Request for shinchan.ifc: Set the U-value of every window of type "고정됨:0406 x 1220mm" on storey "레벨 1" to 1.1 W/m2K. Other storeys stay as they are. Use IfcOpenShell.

First a look at what the model holds.

```python
import ifcopenshell
import ifcopenshell.util.element

model = ifcopenshell.open("shinchan.ifc")
print(model.schema)
storey = next(s for s in model.by_type("IfcBuildingStorey") if s.Name == "레벨 1")
windows = [e for e in ifcopenshell.util.element.get_decomposition(storey) if e.is_a("IfcWindow")]
seen = {}
for e in windows:
    element_type = ifcopenshell.util.element.get_type(e)
    key = (element_type.Name if element_type != e and element_type else None, ifcopenshell.util.element.get_pset(e, "Pset_WindowCommon", "ThermalTransmittance"))
    seen[key] = seen.get(key, 0) + 1
for (name, value), count in sorted(seen.items(), key=str):
    print(count, "x", name, "|", value)
```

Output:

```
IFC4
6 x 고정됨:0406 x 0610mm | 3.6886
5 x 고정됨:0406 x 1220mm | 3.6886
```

```python
import ifcopenshell
import ifcopenshell.api.pset
import ifcopenshell.util.element

model = ifcopenshell.open("shinchan.ifc")

storey = next(s for s in model.by_type("IfcBuildingStorey") if s.Name == "레벨 1")
windows = [e for e in ifcopenshell.util.element.get_decomposition(storey) if e.is_a("IfcWindow")]

count = 0
for e in windows:
    element_type = ifcopenshell.util.element.get_type(e)
    if element_type in (None, e) or element_type.Name != "고정됨:0406 x 1220mm":
        continue
    # add_pset returns the element's existing set when there is one.
    pset = ifcopenshell.api.pset.add_pset(model, product=e, name="Pset_WindowCommon")
    ifcopenshell.api.pset.edit_pset(model, pset=pset, properties={"ThermalTransmittance": 1.1})
    count += 1

print(count, "windows updated")

model.write("shinchan-out.ifc")
```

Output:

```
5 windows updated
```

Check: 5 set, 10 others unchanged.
